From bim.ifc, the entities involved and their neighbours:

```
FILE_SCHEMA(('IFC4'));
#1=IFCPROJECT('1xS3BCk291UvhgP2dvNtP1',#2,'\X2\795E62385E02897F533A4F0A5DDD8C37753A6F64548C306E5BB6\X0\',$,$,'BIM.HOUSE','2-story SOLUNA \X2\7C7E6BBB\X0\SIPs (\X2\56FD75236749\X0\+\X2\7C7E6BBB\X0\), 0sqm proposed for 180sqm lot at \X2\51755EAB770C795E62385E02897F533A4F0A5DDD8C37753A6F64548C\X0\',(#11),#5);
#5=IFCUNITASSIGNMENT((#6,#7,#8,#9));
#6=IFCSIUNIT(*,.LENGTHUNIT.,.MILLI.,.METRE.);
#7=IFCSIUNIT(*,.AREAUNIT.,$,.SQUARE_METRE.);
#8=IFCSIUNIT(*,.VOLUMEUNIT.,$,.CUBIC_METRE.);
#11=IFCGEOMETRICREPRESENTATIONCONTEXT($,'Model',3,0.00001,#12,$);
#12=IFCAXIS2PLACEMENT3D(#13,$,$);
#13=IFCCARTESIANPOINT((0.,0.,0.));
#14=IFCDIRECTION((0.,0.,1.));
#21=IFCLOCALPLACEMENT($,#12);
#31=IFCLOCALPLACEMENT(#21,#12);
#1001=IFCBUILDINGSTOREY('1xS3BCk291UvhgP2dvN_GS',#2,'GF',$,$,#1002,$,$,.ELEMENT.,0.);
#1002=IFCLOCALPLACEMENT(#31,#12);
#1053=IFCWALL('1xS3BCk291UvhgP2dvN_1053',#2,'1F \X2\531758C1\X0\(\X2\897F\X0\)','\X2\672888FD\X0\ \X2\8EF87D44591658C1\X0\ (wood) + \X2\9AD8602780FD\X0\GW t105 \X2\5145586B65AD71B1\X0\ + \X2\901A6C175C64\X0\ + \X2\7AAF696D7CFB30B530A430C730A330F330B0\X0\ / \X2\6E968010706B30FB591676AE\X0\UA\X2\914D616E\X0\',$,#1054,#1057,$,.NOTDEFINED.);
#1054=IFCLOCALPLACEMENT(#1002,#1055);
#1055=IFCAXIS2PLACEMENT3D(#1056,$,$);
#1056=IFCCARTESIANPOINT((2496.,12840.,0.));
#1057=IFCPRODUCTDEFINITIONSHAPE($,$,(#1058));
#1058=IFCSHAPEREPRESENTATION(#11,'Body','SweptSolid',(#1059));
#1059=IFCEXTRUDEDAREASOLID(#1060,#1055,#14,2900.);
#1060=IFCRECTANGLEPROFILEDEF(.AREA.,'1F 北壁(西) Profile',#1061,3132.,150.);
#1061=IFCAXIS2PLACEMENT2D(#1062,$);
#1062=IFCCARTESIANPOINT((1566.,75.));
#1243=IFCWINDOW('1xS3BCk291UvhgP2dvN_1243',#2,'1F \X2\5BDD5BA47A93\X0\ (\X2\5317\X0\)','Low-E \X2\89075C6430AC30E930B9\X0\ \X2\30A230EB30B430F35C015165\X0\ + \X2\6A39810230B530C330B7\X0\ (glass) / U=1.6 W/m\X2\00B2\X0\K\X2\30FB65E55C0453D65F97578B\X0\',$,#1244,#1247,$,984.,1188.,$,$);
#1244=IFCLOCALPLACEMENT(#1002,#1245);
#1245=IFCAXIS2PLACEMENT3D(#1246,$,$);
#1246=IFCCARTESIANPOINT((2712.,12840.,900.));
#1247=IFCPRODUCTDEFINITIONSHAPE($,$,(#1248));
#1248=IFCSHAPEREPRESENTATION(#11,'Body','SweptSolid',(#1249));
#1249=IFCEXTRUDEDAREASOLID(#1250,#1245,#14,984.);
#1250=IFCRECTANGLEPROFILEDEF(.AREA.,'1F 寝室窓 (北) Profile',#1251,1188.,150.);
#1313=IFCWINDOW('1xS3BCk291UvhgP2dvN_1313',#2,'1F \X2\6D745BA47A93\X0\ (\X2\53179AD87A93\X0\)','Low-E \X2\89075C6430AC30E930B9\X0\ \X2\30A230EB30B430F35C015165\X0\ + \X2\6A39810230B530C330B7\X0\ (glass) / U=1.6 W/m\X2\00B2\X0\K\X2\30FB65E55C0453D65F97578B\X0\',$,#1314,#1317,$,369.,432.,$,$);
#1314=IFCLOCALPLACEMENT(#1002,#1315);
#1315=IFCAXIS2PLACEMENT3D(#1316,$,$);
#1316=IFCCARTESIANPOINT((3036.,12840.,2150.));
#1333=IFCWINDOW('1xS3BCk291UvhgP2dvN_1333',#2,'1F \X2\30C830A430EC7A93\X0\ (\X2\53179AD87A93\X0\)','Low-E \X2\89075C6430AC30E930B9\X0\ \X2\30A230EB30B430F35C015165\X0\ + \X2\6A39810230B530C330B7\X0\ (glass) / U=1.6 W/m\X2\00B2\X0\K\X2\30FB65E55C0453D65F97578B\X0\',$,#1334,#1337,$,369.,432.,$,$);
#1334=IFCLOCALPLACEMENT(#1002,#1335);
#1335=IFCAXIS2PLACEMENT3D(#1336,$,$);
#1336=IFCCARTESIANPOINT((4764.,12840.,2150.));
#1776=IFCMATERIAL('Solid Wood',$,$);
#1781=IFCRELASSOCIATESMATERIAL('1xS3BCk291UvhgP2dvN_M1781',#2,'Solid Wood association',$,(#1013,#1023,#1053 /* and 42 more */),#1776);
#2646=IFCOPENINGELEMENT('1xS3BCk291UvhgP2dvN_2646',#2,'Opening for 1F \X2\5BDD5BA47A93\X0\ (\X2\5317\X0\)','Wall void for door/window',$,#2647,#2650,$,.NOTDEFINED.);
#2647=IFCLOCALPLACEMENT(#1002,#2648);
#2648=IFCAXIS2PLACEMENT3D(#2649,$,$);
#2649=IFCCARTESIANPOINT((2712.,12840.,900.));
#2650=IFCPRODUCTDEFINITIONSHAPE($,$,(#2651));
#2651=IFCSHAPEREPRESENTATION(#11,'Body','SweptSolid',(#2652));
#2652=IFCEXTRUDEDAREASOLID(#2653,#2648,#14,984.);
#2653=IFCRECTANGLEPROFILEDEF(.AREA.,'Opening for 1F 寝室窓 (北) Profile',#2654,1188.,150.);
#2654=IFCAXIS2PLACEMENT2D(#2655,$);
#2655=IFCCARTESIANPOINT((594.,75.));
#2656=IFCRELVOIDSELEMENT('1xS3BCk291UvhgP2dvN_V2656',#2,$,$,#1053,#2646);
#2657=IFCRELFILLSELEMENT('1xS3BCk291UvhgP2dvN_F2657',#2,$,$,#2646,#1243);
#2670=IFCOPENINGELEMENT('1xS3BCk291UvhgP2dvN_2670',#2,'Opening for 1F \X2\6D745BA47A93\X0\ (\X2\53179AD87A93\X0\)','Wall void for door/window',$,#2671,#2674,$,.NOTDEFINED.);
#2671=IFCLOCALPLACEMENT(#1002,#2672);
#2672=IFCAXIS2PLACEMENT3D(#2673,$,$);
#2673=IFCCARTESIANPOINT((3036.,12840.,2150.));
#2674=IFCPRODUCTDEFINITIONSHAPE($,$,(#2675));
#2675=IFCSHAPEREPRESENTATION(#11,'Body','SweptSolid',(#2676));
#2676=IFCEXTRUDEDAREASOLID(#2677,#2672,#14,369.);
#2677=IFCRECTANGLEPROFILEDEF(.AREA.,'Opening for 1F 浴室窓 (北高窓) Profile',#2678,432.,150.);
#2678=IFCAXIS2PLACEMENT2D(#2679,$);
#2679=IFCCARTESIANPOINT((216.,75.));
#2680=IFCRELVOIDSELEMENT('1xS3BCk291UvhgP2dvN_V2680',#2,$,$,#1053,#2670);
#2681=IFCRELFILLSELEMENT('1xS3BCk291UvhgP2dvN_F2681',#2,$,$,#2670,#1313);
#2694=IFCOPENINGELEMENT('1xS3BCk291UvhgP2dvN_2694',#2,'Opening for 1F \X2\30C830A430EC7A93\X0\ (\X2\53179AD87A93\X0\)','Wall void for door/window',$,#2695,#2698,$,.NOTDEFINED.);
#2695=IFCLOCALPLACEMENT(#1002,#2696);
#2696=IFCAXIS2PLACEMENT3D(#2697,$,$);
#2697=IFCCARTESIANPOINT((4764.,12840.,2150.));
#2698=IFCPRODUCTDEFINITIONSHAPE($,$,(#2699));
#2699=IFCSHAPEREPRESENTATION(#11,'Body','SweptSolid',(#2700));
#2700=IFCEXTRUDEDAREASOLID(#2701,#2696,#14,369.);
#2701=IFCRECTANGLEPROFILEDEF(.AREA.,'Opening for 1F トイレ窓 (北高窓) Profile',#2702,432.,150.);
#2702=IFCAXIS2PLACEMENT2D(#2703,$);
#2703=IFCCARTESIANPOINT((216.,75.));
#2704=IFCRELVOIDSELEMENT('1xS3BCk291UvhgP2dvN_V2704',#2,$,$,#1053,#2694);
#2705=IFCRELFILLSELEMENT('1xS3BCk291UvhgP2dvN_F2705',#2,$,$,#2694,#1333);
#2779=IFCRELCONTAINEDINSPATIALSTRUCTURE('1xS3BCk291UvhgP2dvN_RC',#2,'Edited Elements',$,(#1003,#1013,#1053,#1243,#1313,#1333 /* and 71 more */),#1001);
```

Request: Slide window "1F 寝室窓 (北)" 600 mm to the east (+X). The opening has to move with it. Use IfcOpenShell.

```python
import ifcopenshell
import ifcopenshell.api.geometry
import ifcopenshell.util.placement

model = ifcopenshell.open("bim.ifc")

window = model.by_guid("1xS3BCk291UvhgP2dvN_1243")
opening = window.FillsVoids[0].RelatingOpeningElement
wall = opening.VoidsElements[0].RelatingBuildingElement

wall_matrix = ifcopenshell.util.placement.get_local_placement(wall.ObjectPlacement)
shift = wall_matrix[:3, 0] * 600.0
before = ifcopenshell.util.placement.get_local_placement(window.ObjectPlacement)[:3, 3].copy()

# The window is not placed relative to its opening, so move both.
for product in (opening, window):
    matrix = ifcopenshell.util.placement.get_local_placement(product.ObjectPlacement)
    matrix[:3, 3] += shift
    ifcopenshell.api.geometry.edit_object_placement(model, product=product, matrix=matrix, is_si=False)

after = ifcopenshell.util.placement.get_local_placement(window.ObjectPlacement)[:3, 3]
print("window moved by", (after - before).round(3) + 0.0)

model.write("bim_rev.ifc")
```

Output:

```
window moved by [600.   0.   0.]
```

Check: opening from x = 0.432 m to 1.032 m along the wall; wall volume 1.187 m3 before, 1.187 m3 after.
